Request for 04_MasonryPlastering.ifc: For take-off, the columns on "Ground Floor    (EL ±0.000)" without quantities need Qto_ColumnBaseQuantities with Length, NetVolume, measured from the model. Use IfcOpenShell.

First a look at what the model holds.

```python
import ifcopenshell
import ifcopenshell.util.element
import ifcopenshell.util.unit

model = ifcopenshell.open("04_MasonryPlastering.ifc")
print(model.schema)
for unit_type in ("LENGTHUNIT", "AREAUNIT", "VOLUMEUNIT"):
    print(unit_type, ifcopenshell.util.unit.calculate_unit_scale(model, unit_type))
storey = next(s for s in model.by_type("IfcBuildingStorey") if s.Name == "Ground Floor    (EL ±0.000)")
columns = [e for e in ifcopenshell.util.element.get_decomposition(storey) if e.is_a("IfcColumn")]
for e in sorted(columns, key=lambda e: e.id()):
    print(e.id(), e.is_a(), e.Name, list(ifcopenshell.util.element.get_psets(e, qtos_only=True)), sep=" | ")
```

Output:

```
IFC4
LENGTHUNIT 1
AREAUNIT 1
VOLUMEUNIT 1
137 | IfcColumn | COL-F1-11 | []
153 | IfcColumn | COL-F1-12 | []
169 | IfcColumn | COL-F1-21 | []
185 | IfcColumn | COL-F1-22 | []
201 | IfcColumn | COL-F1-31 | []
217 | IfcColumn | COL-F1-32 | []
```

```python
import ifcopenshell
import ifcopenshell.api.pset
import ifcopenshell.geom
import ifcopenshell.util.element
import ifcopenshell.util.shape
import ifcopenshell.util.unit

model = ifcopenshell.open("04_MasonryPlastering.ifc")
unit_scale = ifcopenshell.util.unit.calculate_unit_scale(model)
volume_scale = ifcopenshell.util.unit.calculate_unit_scale(model, "VOLUMEUNIT")
settings = ifcopenshell.geom.settings()

storey = next(s for s in model.by_type("IfcBuildingStorey") if s.Name == "Ground Floor    (EL ±0.000)")
columns = [e for e in ifcopenshell.util.element.get_decomposition(storey) if e.is_a("IfcColumn")]

for e in sorted(columns, key=lambda e: e.id()):
    if ifcopenshell.util.element.get_psets(e, qtos_only=True, should_inherit=False):
        continue
    # Geometry comes back in metres, in the element's own axes.
    shape = ifcopenshell.geom.create_shape(settings, e)
    values = {
        "Length": ifcopenshell.util.shape.get_z(shape.geometry) / unit_scale,
        "NetVolume": ifcopenshell.util.shape.get_volume(shape.geometry) / volume_scale,
    }
    qto = ifcopenshell.api.pset.add_qto(model, product=e, name="Qto_ColumnBaseQuantities")
    ifcopenshell.api.pset.edit_qto(model, qto=qto, properties=values)
    print(e.id(), {k: round(v, 3) for k, v in values.items()})

model.write("04_MasonryPlastering_edited.ifc")
```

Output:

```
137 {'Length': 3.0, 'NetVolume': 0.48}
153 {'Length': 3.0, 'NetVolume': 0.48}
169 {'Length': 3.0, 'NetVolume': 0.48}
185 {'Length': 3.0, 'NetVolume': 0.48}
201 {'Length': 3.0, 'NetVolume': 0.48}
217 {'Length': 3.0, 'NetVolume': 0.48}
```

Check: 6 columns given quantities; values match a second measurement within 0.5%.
